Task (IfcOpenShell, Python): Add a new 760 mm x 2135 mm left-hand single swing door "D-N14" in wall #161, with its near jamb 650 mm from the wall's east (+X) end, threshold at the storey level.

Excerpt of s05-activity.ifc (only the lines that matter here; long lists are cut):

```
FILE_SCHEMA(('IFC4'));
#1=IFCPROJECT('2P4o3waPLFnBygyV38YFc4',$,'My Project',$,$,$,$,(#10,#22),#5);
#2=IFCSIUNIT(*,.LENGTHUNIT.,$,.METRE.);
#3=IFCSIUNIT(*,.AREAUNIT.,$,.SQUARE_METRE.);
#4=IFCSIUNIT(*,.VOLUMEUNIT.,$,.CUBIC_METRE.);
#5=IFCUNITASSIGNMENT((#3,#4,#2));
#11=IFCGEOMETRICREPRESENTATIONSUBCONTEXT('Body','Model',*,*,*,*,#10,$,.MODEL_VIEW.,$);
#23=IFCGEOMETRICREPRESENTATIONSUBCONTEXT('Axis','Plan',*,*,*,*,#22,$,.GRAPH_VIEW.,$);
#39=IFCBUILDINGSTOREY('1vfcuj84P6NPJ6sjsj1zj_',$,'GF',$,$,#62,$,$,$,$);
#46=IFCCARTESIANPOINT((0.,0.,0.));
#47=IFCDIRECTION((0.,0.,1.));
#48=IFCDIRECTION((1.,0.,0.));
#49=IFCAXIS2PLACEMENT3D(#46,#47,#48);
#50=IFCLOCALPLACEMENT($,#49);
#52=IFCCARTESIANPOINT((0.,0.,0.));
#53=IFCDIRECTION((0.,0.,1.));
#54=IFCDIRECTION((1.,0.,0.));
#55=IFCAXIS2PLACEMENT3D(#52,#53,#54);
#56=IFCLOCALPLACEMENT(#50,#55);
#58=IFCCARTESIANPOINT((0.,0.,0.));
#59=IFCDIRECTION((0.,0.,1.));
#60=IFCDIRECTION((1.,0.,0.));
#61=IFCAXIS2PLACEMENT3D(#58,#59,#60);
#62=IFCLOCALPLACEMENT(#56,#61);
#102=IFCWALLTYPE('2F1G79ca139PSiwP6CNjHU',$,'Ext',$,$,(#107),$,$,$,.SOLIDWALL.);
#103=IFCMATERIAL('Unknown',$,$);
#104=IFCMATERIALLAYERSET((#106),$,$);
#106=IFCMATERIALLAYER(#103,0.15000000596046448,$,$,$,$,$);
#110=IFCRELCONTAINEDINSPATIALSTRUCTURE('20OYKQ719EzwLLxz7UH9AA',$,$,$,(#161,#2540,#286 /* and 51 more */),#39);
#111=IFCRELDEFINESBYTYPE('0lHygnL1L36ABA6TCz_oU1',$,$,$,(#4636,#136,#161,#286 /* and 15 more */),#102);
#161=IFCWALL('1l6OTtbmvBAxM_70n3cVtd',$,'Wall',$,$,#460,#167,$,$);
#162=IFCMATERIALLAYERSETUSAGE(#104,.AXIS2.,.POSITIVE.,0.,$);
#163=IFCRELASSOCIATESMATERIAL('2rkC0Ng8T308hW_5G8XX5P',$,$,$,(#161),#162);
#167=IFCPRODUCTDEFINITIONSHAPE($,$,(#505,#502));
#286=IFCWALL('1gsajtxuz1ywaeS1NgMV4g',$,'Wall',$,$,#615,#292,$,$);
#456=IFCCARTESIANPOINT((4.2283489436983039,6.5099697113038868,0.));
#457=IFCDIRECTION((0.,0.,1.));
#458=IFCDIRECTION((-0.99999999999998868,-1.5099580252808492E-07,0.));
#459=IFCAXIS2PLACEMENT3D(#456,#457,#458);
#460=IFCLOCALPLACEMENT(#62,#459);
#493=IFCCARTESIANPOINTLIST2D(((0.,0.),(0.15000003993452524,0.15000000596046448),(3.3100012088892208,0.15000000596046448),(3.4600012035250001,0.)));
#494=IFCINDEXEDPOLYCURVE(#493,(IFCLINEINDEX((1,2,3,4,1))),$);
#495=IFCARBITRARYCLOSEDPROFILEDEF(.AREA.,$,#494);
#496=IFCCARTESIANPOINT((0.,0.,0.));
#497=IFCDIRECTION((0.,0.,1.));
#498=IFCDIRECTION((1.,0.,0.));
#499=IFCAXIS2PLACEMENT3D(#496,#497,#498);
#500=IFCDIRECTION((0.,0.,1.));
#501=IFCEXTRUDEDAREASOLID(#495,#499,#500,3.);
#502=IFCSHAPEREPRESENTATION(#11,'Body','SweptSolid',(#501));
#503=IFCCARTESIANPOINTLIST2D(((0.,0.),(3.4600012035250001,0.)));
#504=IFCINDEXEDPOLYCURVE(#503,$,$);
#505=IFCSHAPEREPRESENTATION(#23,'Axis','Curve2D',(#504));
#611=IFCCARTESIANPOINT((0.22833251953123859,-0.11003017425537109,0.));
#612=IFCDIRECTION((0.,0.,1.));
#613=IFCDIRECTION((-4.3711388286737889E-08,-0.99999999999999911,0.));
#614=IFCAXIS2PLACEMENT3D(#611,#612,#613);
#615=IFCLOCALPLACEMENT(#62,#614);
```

```python
import numpy as np
import ifcopenshell
import ifcopenshell.api.feature
import ifcopenshell.api.geometry
import ifcopenshell.api.root
import ifcopenshell.api.spatial
import ifcopenshell.geom
import ifcopenshell.util.element
import ifcopenshell.util.placement
import ifcopenshell.util.representation
import ifcopenshell.util.shape
import ifcopenshell.util.unit

model = ifcopenshell.open("s05-activity.ifc")
unit_scale = ifcopenshell.util.unit.calculate_unit_scale(model)
settings = ifcopenshell.geom.settings()


def volume(element):
    """Net volume in cubic metres, openings subtracted."""
    shape = ifcopenshell.geom.create_shape(settings, element)
    return ifcopenshell.util.shape.get_volume(shape.geometry)


wall = model.by_id(161)
storey = ifcopenshell.util.element.get_container(wall, ifc_class="IfcBuildingStorey")
context = ifcopenshell.util.representation.get_context(model, "Model", "Body", "MODEL_VIEW")
before = volume(wall)

width, height, from_end, sill = 0.76, 2.135, 0.65, 0.0  # metres

# The wall runs along its own X axis, and the end named is its -X end.
wall_shape = ifcopenshell.geom.create_shape(settings, wall)
x, y, z = ifcopenshell.util.shape.get_vertices(wall_shape.geometry).T
start = x.min() + from_end
face, thickness = float(y.min()), float(y.max() - y.min())
wall_matrix = ifcopenshell.util.placement.get_local_placement(wall.ObjectPlacement)
level = ifcopenshell.util.placement.get_local_placement(storey.ObjectPlacement)[2, 3]


def in_wall(x, y):
    """Placement at x, y metres in the wall's axes, at sill height."""
    matrix = wall_matrix.copy()
    matrix[:, 3] = wall_matrix @ np.array([x / unit_scale, y / unit_scale, 0.0, 1.0])
    matrix[2, 3] = level + sill / unit_scale
    return matrix


# Opening: a box that overshoots both wall faces by 50 mm.
opening = ifcopenshell.api.root.create_entity(model, ifc_class="IfcOpeningElement", predefined_type="OPENING")
box = ifcopenshell.api.geometry.add_wall_representation(
    model, context=context, length=width, height=height, thickness=thickness + 0.1
)
ifcopenshell.api.geometry.assign_representation(model, product=opening, representation=box)
ifcopenshell.api.geometry.edit_object_placement(model, product=opening, matrix=in_wall(start, face - 0.05), is_si=False)
ifcopenshell.api.feature.add_feature(model, feature=opening, element=wall)

door = ifcopenshell.api.root.create_entity(model, ifc_class="IfcDoor", name="D-N14", predefined_type="DOOR")
door.OverallWidth, door.OverallHeight = width / unit_scale, height / unit_scale
door.OperationType = "SINGLE_SWING_LEFT"
body = ifcopenshell.api.geometry.add_door_representation(
    model,
    context=context,
    overall_width=door.OverallWidth,
    overall_height=door.OverallHeight,
    operation_type="SINGLE_SWING_LEFT",
    lining_properties={"LiningDepth": thickness / unit_scale, "ThresholdDepth": thickness / unit_scale},
)
ifcopenshell.api.geometry.assign_representation(model, product=door, representation=body)
ifcopenshell.api.spatial.assign_container(model, products=[door], relating_structure=storey)
ifcopenshell.api.feature.add_filling(model, opening=opening, element=door)

# The lining spans the wall, so the door starts at the wall face.
ifcopenshell.api.geometry.edit_object_placement(model, product=door, matrix=in_wall(start, face), is_si=False)

after = volume(wall)

print(f"wall volume {before:.3f} -> {after:.3f} m3")

model.write("s05-activity_updated.ifc")
```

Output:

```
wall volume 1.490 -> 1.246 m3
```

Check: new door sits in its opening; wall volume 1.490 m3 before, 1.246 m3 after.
